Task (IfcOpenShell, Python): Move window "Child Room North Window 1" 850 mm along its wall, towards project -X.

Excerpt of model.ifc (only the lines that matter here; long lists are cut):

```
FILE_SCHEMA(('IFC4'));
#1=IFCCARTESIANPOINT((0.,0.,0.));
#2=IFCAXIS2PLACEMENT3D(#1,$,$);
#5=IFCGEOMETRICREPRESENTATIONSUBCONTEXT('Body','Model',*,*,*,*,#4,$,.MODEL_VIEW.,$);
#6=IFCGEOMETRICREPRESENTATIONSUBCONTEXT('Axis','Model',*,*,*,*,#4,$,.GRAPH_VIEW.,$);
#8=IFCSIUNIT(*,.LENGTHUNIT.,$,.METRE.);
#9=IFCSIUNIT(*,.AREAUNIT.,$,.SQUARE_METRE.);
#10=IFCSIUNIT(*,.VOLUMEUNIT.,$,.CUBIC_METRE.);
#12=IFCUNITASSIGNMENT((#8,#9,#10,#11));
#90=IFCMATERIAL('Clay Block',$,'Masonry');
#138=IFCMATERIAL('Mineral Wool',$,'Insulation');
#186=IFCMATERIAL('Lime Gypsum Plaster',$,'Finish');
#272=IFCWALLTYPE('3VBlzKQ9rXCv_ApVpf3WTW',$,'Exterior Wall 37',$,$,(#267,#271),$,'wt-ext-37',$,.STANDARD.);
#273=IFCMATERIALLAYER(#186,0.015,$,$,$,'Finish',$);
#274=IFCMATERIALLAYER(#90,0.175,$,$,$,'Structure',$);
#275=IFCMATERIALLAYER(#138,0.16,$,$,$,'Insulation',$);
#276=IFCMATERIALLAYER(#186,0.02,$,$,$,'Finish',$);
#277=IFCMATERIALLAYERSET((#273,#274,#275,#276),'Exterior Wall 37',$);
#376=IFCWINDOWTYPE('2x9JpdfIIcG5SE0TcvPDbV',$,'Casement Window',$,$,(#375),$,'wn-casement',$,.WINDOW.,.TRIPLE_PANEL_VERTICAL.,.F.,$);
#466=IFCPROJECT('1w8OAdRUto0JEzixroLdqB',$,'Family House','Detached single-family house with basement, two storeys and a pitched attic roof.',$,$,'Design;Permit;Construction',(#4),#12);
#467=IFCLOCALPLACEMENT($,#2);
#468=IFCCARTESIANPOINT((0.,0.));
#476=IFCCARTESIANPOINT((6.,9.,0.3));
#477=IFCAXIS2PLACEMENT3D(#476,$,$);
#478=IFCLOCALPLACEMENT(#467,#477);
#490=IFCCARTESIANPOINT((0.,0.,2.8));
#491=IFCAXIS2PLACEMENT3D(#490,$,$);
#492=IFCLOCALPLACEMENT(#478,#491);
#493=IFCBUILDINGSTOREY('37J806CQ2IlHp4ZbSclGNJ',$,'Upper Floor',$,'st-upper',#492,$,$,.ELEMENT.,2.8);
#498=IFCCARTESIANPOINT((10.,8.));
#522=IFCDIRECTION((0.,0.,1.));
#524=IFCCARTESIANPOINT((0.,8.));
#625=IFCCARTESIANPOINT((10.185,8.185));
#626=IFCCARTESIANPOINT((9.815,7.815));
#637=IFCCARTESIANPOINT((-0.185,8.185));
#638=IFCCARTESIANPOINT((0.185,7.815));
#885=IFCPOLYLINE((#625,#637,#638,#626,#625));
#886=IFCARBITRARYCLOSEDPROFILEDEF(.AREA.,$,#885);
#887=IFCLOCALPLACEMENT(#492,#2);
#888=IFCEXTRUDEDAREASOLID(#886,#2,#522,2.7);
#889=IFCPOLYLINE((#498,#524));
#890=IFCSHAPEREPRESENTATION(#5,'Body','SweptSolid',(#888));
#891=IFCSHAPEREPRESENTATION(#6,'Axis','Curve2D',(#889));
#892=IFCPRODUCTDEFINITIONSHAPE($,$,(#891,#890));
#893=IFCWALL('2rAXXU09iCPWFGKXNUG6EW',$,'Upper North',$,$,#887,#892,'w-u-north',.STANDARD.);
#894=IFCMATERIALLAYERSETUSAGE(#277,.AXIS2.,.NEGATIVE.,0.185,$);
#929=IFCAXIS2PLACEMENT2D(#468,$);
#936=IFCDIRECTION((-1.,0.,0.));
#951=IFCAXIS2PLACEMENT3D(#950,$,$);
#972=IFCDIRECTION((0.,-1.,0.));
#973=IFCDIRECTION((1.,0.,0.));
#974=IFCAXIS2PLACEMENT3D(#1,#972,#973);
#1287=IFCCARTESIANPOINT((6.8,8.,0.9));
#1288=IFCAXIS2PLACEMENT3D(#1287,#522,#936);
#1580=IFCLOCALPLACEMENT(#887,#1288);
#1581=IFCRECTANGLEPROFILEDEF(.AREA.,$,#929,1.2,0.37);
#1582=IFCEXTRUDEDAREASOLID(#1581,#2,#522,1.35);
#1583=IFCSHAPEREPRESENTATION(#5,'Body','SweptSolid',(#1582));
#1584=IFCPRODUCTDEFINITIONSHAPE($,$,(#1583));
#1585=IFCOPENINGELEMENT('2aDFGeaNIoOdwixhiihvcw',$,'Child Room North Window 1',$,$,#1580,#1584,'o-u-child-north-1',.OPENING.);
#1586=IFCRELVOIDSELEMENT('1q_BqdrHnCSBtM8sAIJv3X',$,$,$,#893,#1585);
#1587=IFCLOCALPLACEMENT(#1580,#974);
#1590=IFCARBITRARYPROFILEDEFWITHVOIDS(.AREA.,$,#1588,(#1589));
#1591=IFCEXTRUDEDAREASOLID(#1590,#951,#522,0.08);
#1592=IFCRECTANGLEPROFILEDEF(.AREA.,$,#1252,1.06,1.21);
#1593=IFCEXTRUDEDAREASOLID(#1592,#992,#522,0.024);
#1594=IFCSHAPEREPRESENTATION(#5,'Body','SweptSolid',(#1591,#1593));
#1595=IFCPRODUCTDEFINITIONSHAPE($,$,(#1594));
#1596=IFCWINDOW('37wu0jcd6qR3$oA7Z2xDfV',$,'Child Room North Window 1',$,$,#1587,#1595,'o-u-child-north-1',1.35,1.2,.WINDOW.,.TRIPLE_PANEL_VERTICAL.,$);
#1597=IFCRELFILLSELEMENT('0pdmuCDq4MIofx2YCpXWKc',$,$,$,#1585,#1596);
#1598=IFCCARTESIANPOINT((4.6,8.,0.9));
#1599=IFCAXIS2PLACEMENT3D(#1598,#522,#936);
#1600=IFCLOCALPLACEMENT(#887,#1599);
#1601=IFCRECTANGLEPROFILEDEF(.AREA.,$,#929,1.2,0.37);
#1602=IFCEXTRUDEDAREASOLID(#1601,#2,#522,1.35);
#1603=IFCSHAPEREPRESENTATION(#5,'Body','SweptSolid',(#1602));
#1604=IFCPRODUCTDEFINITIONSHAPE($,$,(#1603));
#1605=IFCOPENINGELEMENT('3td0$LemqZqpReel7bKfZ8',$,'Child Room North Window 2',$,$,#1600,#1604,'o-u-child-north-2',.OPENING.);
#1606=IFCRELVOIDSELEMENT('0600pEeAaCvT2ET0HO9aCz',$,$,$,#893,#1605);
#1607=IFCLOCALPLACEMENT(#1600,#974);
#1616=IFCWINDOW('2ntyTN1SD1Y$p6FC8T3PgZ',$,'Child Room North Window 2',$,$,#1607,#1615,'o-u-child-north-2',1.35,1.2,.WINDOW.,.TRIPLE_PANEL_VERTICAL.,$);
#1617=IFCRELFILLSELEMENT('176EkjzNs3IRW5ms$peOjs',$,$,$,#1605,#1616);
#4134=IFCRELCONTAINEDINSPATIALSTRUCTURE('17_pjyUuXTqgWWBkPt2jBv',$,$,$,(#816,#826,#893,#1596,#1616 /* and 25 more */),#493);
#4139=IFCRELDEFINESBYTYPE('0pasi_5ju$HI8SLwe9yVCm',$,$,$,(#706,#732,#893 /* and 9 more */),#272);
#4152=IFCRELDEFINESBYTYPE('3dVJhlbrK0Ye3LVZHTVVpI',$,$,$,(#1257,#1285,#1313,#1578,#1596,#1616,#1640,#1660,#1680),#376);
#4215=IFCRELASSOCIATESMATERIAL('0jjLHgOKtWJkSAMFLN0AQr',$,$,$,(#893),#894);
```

```python
import ifcopenshell
import ifcopenshell.api.geometry
import ifcopenshell.util.placement
import ifcopenshell.util.unit

model = ifcopenshell.open("model.ifc")
unit_scale = ifcopenshell.util.unit.calculate_unit_scale(model)

window = model.by_guid("37wu0jcd6qR3$oA7Z2xDfV")
opening = window.FillsVoids[0].RelatingOpeningElement
wall = opening.VoidsElements[0].RelatingBuildingElement

wall_matrix = ifcopenshell.util.placement.get_local_placement(wall.ObjectPlacement)
shift = wall_matrix[:3, 0] * -0.85 / unit_scale
before = ifcopenshell.util.placement.get_local_placement(window.ObjectPlacement)[:3, 3].copy()

# The window is placed relative to its opening, so it follows when the opening moves.
matrix = ifcopenshell.util.placement.get_local_placement(opening.ObjectPlacement)
matrix[:3, 3] += shift
ifcopenshell.api.geometry.edit_object_placement(
    model, product=opening, matrix=matrix, is_si=False, should_transform_children=True
)

after = ifcopenshell.util.placement.get_local_placement(window.ObjectPlacement)[:3, 3]
print("window moved by", (after - before).round(3) + 0.0)

model.write("model_updated.ifc")
```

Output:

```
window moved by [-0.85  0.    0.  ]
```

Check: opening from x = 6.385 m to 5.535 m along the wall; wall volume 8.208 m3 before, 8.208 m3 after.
